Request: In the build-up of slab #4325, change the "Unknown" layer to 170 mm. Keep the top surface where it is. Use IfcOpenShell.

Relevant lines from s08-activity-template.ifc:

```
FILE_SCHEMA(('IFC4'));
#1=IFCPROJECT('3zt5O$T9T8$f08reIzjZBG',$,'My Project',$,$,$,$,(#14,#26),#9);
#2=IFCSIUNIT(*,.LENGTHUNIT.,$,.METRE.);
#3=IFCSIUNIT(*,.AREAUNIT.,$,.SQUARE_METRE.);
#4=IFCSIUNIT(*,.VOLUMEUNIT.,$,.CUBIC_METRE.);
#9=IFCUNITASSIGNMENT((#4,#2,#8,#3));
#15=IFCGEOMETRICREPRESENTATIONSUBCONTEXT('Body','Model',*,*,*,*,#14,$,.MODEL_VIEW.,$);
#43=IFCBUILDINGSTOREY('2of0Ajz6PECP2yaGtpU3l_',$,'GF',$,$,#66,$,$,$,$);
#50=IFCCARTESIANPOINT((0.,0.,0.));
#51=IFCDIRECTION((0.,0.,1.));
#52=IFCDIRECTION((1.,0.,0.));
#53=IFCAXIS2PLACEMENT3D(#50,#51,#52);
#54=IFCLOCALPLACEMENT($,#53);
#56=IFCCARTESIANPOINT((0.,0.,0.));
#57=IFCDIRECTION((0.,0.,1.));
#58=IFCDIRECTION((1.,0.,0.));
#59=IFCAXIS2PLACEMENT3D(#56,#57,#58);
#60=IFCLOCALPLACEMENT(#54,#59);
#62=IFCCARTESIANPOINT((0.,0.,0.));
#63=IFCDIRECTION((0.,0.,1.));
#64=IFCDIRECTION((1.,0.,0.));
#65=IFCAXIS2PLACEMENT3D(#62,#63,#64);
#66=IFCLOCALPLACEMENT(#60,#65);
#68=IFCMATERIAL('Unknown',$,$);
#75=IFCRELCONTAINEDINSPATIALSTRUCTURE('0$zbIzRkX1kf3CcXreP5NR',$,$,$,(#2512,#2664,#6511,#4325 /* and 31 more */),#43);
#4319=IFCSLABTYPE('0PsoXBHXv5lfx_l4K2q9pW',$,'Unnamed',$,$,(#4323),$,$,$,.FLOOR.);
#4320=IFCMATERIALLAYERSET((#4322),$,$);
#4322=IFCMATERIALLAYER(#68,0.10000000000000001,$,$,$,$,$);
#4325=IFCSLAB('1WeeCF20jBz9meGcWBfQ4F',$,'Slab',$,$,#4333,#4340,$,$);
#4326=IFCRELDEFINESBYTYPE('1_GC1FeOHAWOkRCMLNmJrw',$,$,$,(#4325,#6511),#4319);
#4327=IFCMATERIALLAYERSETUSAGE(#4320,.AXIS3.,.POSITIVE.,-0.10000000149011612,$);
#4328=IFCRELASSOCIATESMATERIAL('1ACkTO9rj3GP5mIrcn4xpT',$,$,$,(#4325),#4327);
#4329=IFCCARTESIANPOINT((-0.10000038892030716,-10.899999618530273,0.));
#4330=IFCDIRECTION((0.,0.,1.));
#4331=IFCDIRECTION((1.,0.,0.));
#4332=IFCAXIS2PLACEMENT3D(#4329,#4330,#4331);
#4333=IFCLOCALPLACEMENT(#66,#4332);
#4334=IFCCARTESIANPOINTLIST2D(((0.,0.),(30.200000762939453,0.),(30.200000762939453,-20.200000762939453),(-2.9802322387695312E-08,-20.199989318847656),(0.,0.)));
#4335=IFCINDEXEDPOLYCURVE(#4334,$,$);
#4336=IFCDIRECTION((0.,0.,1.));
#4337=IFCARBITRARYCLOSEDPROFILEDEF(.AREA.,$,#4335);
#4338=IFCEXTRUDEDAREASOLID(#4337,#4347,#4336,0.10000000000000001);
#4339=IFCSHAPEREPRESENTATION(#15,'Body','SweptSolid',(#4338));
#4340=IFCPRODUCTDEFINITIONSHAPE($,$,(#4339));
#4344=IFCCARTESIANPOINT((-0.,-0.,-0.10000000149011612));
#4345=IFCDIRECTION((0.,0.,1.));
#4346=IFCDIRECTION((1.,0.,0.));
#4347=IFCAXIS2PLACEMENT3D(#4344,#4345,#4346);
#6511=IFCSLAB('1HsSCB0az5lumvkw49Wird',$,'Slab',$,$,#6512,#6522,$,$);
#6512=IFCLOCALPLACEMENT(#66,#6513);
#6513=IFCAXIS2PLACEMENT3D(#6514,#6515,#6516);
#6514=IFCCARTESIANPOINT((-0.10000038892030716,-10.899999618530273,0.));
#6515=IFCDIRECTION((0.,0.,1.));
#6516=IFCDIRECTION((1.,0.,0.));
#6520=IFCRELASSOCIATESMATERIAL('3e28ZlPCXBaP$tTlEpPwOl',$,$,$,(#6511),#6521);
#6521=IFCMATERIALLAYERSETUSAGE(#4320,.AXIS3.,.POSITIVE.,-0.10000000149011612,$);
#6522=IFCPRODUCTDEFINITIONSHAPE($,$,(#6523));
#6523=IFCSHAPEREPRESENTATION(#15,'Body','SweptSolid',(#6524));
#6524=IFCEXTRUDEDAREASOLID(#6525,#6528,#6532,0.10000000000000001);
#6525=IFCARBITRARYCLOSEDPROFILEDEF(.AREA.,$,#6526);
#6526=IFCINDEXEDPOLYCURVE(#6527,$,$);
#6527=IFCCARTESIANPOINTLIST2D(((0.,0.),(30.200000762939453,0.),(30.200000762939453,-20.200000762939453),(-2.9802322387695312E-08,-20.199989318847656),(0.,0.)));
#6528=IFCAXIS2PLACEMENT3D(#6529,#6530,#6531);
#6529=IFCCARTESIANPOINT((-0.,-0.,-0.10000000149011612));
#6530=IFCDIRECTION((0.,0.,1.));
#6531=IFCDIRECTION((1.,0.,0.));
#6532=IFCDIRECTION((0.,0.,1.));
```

```python
import ifcopenshell
import ifcopenshell.util.element
import ifcopenshell.util.representation
import ifcopenshell.util.unit

model = ifcopenshell.open("s08-activity-template.ifc")
unit_scale = ifcopenshell.util.unit.calculate_unit_scale(model)

layer_set = model.by_id(4320)
layer = next(l for l in layer_set.MaterialLayers if l.Material and l.Material.Name == "Unknown")
change = 0.17 / unit_scale - layer.LayerThickness
layer.LayerThickness += change

# The layer set is shared, so every slab that uses it gets the new thickness.
slabs = [e for e in ifcopenshell.util.element.get_elements_by_material(model, layer_set) if e.is_a("IfcSlab")]
for slab in sorted(slabs, key=lambda e: e.id()):
    body = ifcopenshell.util.representation.get_representation(slab, "Model", "Body")
    solid = body.Items[0]
    old_depth = solid.Depth
    solid.Depth += change
    # Extruded upwards: lower the start of the extrusion so the top stays.
    x, y, z = solid.Position.Location.Coordinates
    solid.Position.Location = model.createIfcCartesianPoint((x, y, z - change))
    print(slab.id(), f"{old_depth:g} -> {solid.Depth:g}")

# The layers are counted up from the underside, which has moved.
for usage in {ifcopenshell.util.element.get_material(slab) for slab in slabs}:
    usage.OffsetFromReferenceLine -= change

model.write("s08-activity-template_edited.ifc")
```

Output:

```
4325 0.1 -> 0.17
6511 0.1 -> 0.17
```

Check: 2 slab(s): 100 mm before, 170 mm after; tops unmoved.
